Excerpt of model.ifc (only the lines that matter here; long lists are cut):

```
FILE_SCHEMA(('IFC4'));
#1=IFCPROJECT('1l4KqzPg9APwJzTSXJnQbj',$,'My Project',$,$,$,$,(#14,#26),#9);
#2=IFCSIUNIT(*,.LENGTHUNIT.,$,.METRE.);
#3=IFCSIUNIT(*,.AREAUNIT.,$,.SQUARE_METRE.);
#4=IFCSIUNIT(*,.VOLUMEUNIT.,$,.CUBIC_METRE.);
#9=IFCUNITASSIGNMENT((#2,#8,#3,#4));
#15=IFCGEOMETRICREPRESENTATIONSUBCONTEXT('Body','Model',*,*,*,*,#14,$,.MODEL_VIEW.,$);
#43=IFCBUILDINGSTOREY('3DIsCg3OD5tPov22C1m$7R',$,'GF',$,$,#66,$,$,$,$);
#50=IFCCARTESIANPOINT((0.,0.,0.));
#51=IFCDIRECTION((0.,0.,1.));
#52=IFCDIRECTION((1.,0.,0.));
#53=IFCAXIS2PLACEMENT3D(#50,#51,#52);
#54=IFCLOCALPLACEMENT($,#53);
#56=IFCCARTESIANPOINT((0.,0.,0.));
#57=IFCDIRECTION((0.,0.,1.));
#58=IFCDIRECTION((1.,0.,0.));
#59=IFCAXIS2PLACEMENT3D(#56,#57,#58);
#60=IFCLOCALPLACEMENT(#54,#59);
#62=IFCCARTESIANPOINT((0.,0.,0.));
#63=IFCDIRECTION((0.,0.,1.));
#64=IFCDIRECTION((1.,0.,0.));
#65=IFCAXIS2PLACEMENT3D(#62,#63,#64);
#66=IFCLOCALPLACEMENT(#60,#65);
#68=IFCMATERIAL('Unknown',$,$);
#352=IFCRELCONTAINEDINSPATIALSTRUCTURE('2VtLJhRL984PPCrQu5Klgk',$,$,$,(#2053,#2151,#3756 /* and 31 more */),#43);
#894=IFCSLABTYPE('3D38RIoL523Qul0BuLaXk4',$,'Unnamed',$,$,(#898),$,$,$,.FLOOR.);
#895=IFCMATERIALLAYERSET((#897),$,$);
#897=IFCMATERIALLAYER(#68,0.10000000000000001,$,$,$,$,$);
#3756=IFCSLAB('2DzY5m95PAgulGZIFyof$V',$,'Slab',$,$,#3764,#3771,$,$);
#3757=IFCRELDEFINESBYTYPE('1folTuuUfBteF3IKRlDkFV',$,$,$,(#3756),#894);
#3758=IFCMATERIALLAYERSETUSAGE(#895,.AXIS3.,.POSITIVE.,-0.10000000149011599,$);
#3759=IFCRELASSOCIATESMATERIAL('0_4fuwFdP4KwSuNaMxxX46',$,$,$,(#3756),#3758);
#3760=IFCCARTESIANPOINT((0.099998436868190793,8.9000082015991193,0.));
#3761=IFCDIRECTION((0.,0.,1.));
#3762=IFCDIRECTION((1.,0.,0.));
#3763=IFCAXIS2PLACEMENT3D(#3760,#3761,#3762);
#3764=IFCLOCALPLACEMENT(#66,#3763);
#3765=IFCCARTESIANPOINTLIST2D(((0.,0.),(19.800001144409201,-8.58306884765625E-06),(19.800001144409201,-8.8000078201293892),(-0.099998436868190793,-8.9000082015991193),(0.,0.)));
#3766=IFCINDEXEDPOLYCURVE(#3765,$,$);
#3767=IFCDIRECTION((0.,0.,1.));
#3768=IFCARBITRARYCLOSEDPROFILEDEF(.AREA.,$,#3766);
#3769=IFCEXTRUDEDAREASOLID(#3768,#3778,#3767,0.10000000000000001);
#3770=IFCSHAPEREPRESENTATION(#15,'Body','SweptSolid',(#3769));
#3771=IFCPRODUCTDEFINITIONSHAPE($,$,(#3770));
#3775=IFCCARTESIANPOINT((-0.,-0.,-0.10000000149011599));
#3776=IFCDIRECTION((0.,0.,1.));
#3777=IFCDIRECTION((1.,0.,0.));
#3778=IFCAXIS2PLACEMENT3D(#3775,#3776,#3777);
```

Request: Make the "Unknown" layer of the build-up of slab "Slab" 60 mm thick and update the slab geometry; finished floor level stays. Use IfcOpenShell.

```python
import ifcopenshell
import ifcopenshell.util.element
import ifcopenshell.util.representation
import ifcopenshell.util.unit

model = ifcopenshell.open("model.ifc")
unit_scale = ifcopenshell.util.unit.calculate_unit_scale(model)

layer_set = model.by_id(895)
layer = next(l for l in layer_set.MaterialLayers if l.Material and l.Material.Name == "Unknown")
change = 0.06 / unit_scale - layer.LayerThickness
layer.LayerThickness += change

# Geometry does not follow the layer set by itself.
slabs = [e for e in ifcopenshell.util.element.get_elements_by_material(model, layer_set) if e.is_a("IfcSlab")]
for slab in sorted(slabs, key=lambda e: e.id()):
    body = ifcopenshell.util.representation.get_representation(slab, "Model", "Body")
    solid = body.Items[0]
    old_depth = solid.Depth
    solid.Depth += change
    # Extruded upwards: lower the start of the extrusion so the top stays.
    x, y, z = solid.Position.Location.Coordinates
    solid.Position.Location = model.createIfcCartesianPoint((x, y, z - change))
    print(slab.id(), f"{old_depth:g} -> {solid.Depth:g}")

# The layers are counted up from the underside, which has moved.
for usage in {ifcopenshell.util.element.get_material(slab) for slab in slabs}:
    usage.OffsetFromReferenceLine -= change

model.write("model_edited.ifc")
```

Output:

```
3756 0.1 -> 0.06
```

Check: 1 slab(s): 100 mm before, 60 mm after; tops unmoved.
